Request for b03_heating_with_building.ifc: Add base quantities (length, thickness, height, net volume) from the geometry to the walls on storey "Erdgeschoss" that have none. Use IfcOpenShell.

First a look at what the model holds.

```python
import ifcopenshell
import ifcopenshell.util.element
import ifcopenshell.util.unit

model = ifcopenshell.open("b03_heating_with_building.ifc")
print(model.schema)
for unit_type in ("LENGTHUNIT", "AREAUNIT", "VOLUMEUNIT"):
    print(unit_type, ifcopenshell.util.unit.calculate_unit_scale(model, unit_type))
storey = next(s for s in model.by_type("IfcBuildingStorey") if s.Name == "Erdgeschoss")
walls = [e for e in ifcopenshell.util.element.get_decomposition(storey) if e.is_a("IfcWall")]
for e in sorted(walls, key=lambda e: e.id()):
    print(e.id(), e.is_a(), e.Name, list(ifcopenshell.util.element.get_psets(e, qtos_only=True)), sep=" | ")
```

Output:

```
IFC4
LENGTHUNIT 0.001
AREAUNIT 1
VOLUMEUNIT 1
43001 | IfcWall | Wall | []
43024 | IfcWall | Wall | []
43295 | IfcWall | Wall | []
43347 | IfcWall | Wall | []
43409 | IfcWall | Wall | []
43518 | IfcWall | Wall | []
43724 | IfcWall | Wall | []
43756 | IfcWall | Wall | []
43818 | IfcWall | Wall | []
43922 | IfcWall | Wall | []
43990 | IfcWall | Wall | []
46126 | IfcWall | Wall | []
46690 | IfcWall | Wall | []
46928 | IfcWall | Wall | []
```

```python
import ifcopenshell
import ifcopenshell.api.pset
import ifcopenshell.geom
import ifcopenshell.util.element
import ifcopenshell.util.shape
import ifcopenshell.util.unit

model = ifcopenshell.open("b03_heating_with_building.ifc")
unit_scale = ifcopenshell.util.unit.calculate_unit_scale(model)
volume_scale = ifcopenshell.util.unit.calculate_unit_scale(model, "VOLUMEUNIT")
settings = ifcopenshell.geom.settings()

storey = next(s for s in model.by_type("IfcBuildingStorey") if s.Name == "Erdgeschoss")
walls = [e for e in ifcopenshell.util.element.get_decomposition(storey) if e.is_a("IfcWall")]

for e in sorted(walls, key=lambda e: e.id()):
    if ifcopenshell.util.element.get_psets(e, qtos_only=True, should_inherit=False):
        continue
    # Geometry comes back in metres, in the element's own axes.
    shape = ifcopenshell.geom.create_shape(settings, e)
    values = {
        "Length": ifcopenshell.util.shape.get_x(shape.geometry) / unit_scale,
        "Width": ifcopenshell.util.shape.get_y(shape.geometry) / unit_scale,
        "Height": ifcopenshell.util.shape.get_z(shape.geometry) / unit_scale,
        "NetVolume": ifcopenshell.util.shape.get_volume(shape.geometry) / volume_scale,
    }
    qto = ifcopenshell.api.pset.add_qto(model, product=e, name="Qto_WallBaseQuantities")
    ifcopenshell.api.pset.edit_qto(model, qto=qto, properties=values)
    print(e.id(), {k: round(v, 3) for k, v in values.items()})

model.write("b03_heating_with_building-out.ifc")
```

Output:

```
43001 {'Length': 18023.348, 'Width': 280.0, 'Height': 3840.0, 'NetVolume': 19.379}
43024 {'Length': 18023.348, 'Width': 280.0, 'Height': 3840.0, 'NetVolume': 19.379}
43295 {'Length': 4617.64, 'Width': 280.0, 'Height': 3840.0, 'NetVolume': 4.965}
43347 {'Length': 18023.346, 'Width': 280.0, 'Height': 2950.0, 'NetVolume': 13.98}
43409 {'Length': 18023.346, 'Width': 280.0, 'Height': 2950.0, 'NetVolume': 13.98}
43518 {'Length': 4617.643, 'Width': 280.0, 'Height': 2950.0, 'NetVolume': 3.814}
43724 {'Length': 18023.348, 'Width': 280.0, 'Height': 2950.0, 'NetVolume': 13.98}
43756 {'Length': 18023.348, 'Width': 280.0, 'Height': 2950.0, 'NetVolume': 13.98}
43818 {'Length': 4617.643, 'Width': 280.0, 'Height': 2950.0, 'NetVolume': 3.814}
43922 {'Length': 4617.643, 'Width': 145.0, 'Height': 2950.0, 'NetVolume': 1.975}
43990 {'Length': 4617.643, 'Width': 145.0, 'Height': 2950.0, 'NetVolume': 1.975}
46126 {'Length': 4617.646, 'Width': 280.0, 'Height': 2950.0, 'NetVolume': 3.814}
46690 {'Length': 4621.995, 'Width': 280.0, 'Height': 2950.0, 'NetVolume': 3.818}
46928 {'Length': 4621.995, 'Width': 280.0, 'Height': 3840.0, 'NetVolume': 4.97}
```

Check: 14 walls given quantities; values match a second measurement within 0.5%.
